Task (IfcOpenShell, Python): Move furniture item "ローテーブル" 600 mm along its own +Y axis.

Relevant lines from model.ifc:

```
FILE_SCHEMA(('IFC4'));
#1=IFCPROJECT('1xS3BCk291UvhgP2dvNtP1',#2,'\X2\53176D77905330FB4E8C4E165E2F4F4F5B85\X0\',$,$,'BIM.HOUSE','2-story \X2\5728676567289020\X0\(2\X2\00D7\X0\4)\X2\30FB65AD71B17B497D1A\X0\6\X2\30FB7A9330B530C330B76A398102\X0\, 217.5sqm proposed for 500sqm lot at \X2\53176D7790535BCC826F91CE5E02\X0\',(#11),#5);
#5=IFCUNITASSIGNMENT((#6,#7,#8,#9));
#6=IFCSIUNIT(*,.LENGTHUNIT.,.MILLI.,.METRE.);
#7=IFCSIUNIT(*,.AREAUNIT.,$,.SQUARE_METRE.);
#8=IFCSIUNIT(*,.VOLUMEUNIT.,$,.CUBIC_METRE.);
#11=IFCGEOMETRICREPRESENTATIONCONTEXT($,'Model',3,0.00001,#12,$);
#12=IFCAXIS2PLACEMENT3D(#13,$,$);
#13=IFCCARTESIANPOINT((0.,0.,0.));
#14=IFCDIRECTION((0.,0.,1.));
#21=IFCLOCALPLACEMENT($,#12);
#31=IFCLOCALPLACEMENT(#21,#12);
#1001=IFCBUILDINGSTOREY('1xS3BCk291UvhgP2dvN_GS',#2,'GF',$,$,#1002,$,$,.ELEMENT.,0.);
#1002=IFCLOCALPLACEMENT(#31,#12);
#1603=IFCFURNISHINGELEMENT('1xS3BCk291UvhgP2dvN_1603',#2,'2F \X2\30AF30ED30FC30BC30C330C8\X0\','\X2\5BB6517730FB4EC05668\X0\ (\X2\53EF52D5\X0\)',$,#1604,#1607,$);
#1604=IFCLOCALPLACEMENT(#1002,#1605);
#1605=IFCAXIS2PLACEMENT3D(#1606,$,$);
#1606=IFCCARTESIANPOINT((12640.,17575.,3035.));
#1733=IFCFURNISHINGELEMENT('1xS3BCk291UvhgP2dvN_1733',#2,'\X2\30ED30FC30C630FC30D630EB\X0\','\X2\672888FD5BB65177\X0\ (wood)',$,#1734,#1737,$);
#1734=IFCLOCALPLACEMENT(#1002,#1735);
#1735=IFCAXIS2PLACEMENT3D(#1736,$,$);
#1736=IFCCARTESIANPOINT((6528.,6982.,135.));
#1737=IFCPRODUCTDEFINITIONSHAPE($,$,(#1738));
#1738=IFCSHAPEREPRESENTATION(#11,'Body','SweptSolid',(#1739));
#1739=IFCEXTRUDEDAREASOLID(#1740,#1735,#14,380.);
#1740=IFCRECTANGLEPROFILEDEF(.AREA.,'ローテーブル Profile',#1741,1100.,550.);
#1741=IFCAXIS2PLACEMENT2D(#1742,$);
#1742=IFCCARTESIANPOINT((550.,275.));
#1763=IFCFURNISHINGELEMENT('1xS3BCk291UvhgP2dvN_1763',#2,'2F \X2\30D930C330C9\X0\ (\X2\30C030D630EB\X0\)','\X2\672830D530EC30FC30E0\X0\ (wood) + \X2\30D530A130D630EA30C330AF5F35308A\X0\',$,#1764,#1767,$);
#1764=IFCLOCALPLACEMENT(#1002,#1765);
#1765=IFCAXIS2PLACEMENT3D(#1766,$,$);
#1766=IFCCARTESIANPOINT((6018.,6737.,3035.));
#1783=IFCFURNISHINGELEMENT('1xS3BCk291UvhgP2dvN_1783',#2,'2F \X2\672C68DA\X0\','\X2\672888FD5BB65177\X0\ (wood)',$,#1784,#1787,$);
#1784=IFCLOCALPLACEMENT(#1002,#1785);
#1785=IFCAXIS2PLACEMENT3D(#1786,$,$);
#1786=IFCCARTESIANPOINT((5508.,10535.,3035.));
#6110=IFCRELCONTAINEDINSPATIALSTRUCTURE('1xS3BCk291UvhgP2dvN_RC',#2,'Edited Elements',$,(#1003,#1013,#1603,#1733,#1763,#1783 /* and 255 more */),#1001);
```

```python
import ifcopenshell
import ifcopenshell.api.geometry
import ifcopenshell.util.placement
import ifcopenshell.util.unit

model = ifcopenshell.open("model.ifc")
unit_scale = ifcopenshell.util.unit.calculate_unit_scale(model)

item = model.by_id(1733)
matrix = ifcopenshell.util.placement.get_local_placement(item.ObjectPlacement)
matrix[:3, 3] += matrix[:3, 1] * 0.6 / unit_scale
ifcopenshell.api.geometry.edit_object_placement(model, product=item, matrix=matrix, is_si=False)

print(ifcopenshell.util.placement.get_local_placement(item.ObjectPlacement).round(3) + 0.0)

model.write("model_updated.ifc")
```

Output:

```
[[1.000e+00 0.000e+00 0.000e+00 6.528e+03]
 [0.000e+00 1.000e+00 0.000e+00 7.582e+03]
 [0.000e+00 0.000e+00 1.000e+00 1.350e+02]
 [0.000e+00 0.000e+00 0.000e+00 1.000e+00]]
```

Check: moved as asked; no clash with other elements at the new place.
